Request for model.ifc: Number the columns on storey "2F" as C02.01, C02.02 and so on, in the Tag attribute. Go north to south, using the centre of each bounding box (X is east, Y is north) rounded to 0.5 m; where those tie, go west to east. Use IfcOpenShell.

First a look at what the model holds.

```python
import ifcopenshell
import ifcopenshell.util.element
import ifcopenshell.util.placement

model = ifcopenshell.open("model.ifc")
print(model.schema)
storey = next(s for s in model.by_type("IfcBuildingStorey") if s.Name == "2F")
columns = [e for e in ifcopenshell.util.element.get_decomposition(storey) if e.is_a("IfcColumn")]
for e in sorted(columns, key=lambda e: e.id()):
    origin = ifcopenshell.util.placement.get_local_placement(e.ObjectPlacement)[:3, 3]
    print(e.id(), e.Tag, e.Name, origin.round(2) + 0.0, sep=" | ")
```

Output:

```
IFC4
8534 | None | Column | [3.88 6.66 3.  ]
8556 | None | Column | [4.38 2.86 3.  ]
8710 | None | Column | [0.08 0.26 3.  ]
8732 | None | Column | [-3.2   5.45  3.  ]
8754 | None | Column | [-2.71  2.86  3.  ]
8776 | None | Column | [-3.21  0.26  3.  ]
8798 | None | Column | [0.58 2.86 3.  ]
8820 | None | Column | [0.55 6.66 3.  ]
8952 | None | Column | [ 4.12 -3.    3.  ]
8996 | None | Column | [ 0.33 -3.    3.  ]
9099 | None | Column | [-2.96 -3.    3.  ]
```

```python
import ifcopenshell
import ifcopenshell.geom
import ifcopenshell.util.element
import ifcopenshell.util.shape

model = ifcopenshell.open("model.ifc")
settings = ifcopenshell.geom.settings()
settings.set("use-world-coords", True)


def centre(element):
    shape = ifcopenshell.geom.create_shape(settings, element)
    return ifcopenshell.util.shape.get_bbox_centroid(shape.geometry)


storey = next(s for s in model.by_type("IfcBuildingStorey") if s.Name == "2F")
columns = [e for e in ifcopenshell.util.element.get_decomposition(storey) if e.is_a("IfcColumn")]

# Insertion points can sit at a corner or the storey origin, so sort by the geometry (in metres).
centres = {e: centre(e) for e in columns}
columns.sort(key=lambda e: (-round(centres[e][1] / 0.5), centres[e][0]))

for i, e in enumerate(columns, start=1):
    number = f"C02.{i:02d}"
    e.Tag = number
    print(e.id(), number)

model.write("model-out.ifc")
```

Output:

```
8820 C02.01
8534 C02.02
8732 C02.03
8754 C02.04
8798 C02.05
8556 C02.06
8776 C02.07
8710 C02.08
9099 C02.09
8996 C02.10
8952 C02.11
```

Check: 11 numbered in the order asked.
